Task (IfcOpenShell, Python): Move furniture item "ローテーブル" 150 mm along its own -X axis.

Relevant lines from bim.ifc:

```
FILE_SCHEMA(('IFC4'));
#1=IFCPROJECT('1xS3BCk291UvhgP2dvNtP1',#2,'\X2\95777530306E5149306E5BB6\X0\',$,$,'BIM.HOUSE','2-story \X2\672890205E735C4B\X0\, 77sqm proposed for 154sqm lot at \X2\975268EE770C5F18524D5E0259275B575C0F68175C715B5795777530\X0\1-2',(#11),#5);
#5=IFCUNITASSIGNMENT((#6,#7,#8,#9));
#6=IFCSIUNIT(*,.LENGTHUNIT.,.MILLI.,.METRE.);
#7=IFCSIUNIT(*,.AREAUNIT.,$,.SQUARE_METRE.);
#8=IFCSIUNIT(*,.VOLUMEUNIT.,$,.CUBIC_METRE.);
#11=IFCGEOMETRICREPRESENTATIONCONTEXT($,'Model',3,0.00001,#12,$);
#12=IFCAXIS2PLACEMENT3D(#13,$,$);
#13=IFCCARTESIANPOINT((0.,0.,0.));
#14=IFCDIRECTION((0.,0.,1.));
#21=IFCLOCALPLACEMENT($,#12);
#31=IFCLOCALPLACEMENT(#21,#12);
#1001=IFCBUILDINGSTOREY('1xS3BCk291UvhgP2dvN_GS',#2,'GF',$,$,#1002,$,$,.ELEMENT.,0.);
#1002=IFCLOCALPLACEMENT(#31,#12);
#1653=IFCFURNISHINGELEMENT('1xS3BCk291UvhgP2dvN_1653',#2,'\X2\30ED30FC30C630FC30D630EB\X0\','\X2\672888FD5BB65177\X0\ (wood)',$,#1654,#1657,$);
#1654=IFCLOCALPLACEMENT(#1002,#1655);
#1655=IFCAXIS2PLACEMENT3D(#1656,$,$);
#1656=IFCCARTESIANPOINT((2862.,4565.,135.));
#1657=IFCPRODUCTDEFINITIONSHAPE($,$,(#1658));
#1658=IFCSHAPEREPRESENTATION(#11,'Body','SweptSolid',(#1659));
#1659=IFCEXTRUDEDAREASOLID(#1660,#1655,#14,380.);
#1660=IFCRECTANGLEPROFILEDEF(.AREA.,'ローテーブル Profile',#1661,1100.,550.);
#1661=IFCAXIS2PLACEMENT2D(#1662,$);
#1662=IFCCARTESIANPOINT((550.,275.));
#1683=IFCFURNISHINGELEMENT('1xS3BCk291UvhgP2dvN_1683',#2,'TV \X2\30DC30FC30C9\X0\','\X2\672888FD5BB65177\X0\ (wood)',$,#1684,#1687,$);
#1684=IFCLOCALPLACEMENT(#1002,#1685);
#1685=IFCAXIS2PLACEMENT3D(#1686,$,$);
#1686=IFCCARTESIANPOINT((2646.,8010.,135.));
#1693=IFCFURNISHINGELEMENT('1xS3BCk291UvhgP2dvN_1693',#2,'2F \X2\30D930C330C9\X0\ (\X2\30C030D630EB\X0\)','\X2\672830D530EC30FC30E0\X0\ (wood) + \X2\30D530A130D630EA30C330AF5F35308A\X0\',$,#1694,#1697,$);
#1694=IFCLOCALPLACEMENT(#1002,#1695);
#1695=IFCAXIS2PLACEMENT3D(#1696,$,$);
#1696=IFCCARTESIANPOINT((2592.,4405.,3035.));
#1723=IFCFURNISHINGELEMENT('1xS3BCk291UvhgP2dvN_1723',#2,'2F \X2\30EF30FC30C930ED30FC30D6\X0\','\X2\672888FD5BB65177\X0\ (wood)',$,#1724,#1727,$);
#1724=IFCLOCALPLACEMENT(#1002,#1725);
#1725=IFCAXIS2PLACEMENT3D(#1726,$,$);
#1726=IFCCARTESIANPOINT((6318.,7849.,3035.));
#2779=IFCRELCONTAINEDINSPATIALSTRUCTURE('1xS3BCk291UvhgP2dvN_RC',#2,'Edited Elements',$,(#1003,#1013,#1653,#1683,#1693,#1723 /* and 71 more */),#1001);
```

```python
import ifcopenshell
import ifcopenshell.api.geometry
import ifcopenshell.util.placement
import ifcopenshell.util.unit

model = ifcopenshell.open("bim.ifc")
unit_scale = ifcopenshell.util.unit.calculate_unit_scale(model)

item = model.by_guid("1xS3BCk291UvhgP2dvN_1653")
matrix = ifcopenshell.util.placement.get_local_placement(item.ObjectPlacement)
matrix[:3, 3] -= matrix[:3, 0] * 0.15 / unit_scale
ifcopenshell.api.geometry.edit_object_placement(model, product=item, matrix=matrix, is_si=False)

print(ifcopenshell.util.placement.get_local_placement(item.ObjectPlacement).round(3) + 0.0)

model.write("bim_rev.ifc")
```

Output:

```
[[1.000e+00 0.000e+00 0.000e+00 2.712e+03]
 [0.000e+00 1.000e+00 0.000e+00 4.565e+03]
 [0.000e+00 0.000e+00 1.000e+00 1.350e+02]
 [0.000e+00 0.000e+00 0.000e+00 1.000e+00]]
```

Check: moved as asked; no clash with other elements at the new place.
